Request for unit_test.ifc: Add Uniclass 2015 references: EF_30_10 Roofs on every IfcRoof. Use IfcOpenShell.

First a look at what the model holds.

```python
import ifcopenshell

model = ifcopenshell.open("unit_test.ifc")
print(model.schema)
print("classifications:", [c.Name for c in model.by_type("IfcClassification")])
for ifc_class in ("IfcDoor", "IfcRoof", "IfcStair", "IfcWall", "IfcWindow"):
    print(ifc_class, len(model.by_type(ifc_class)))
```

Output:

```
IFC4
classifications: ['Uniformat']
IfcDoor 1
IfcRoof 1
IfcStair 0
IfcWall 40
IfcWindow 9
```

```python
import ifcopenshell
import ifcopenshell.api.classification

model = ifcopenshell.open("unit_test.ifc")

system = ifcopenshell.api.classification.add_classification(model, classification="Uniclass 2015")

codes = {
    "IfcRoof": ("EF_30_10", "Roofs"),
}
for ifc_class, (code, name) in codes.items():
    products = model.by_type(ifc_class)
    ifcopenshell.api.classification.add_reference(
        model, products=products, classification=system, identification=code, name=name
    )
    print(code, len(products))

model.write("unit_test_updated.ifc")
```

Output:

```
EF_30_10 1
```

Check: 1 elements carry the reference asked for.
